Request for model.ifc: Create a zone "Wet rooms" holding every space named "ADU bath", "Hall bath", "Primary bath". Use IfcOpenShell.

First a look at what the model holds.

```python
import ifcopenshell

model = ifcopenshell.open("model.ifc")
print(model.schema)
seen = {}
for space in model.by_type("IfcSpace"):
    seen[space.Name] = seen.get(space.Name, 0) + 1
for name, count in sorted(seen.items(), key=str):
    print(count, "x", name)
print("zones:", [z.Name for z in model.by_type("IfcZone")][:20])
```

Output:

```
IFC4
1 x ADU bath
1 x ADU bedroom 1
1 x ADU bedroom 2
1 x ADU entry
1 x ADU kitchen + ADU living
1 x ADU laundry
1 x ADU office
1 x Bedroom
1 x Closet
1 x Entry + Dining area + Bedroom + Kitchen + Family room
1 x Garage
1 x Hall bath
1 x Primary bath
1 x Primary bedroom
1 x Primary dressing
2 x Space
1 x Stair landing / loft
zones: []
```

```python
import ifcopenshell
import ifcopenshell.api.group
import ifcopenshell.api.root

model = ifcopenshell.open("model.ifc")

names = {"ADU bath", "Hall bath", "Primary bath"}
spaces = [s for s in model.by_type("IfcSpace") if s.Name in names]

zone = ifcopenshell.api.root.create_entity(model, ifc_class="IfcZone", name="Wet rooms")
ifcopenshell.api.group.assign_group(model, products=spaces, group=zone)
print(len(spaces), "spaces in", zone.Name)

model.write("model_rev.ifc")
```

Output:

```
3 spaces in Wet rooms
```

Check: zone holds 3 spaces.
